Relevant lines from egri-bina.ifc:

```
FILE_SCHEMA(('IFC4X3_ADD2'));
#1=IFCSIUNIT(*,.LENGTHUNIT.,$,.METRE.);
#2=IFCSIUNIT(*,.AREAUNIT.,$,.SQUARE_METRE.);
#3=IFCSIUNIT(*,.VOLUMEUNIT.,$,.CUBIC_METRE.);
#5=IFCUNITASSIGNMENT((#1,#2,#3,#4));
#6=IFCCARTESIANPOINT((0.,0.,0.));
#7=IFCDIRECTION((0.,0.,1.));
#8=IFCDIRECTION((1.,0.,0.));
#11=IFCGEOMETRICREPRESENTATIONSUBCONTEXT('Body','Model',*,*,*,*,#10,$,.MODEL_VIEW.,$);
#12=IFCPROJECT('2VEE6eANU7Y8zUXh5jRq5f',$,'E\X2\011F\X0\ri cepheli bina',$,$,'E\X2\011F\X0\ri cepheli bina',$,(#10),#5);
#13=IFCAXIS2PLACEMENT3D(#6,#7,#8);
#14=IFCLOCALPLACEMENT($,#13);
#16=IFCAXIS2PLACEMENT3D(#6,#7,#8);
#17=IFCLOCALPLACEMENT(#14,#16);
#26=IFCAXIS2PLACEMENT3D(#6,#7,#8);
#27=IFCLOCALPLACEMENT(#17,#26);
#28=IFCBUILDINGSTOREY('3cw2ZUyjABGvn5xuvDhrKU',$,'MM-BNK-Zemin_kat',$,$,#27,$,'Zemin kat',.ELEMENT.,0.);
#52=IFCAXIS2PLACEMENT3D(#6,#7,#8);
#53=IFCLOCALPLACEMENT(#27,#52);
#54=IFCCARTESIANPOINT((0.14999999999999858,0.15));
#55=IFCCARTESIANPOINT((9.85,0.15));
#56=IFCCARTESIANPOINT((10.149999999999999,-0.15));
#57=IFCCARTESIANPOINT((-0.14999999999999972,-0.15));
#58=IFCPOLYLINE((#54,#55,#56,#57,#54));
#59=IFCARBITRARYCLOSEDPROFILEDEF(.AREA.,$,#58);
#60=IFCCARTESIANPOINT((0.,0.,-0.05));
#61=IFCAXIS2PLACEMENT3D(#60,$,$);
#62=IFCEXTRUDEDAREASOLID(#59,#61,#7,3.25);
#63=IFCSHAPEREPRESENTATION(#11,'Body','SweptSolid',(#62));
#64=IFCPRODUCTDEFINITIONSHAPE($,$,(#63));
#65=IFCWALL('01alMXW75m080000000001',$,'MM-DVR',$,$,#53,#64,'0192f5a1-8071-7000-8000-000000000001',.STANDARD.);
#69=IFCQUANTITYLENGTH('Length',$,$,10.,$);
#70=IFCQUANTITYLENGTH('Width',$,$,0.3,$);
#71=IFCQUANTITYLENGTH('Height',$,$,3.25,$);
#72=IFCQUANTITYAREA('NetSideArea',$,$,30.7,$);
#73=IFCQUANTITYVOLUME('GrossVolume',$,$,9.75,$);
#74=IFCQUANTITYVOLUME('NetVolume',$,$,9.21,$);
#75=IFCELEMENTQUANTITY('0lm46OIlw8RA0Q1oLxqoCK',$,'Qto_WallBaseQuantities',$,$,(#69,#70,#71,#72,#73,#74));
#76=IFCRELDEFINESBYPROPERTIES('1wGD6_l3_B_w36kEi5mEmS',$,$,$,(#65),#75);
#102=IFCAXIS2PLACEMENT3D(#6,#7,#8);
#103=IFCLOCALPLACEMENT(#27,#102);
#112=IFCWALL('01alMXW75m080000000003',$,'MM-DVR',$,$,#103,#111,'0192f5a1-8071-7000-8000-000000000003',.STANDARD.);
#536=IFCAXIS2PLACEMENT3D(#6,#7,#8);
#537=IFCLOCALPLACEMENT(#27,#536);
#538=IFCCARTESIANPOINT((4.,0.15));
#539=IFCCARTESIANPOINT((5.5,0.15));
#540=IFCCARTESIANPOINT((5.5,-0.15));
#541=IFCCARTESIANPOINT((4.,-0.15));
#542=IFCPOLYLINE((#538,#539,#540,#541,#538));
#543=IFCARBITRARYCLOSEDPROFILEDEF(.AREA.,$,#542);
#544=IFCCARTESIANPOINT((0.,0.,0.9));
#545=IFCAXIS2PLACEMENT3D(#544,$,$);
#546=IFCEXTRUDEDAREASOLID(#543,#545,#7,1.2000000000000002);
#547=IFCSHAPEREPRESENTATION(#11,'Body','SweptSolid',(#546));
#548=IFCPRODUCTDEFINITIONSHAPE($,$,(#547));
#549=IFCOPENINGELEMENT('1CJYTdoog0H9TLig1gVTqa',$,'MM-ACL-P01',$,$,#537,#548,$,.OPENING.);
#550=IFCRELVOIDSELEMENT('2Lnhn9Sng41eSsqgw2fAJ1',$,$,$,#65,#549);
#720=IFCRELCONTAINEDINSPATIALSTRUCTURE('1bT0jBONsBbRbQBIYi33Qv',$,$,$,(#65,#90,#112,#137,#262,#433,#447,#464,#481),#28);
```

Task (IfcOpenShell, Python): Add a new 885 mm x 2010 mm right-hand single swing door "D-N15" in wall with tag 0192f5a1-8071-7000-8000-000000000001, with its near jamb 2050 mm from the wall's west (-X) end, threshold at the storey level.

```python
import numpy as np
import ifcopenshell
import ifcopenshell.api.feature
import ifcopenshell.api.geometry
import ifcopenshell.api.pset
import ifcopenshell.api.root
import ifcopenshell.api.spatial
import ifcopenshell.geom
import ifcopenshell.util.element
import ifcopenshell.util.placement
import ifcopenshell.util.representation
import ifcopenshell.util.shape
import ifcopenshell.util.unit

model = ifcopenshell.open("egri-bina.ifc")
unit_scale = ifcopenshell.util.unit.calculate_unit_scale(model)
area_scale = ifcopenshell.util.unit.calculate_unit_scale(model, "AREAUNIT")
volume_scale = ifcopenshell.util.unit.calculate_unit_scale(model, "VOLUMEUNIT")
settings = ifcopenshell.geom.settings()


def volume(element):
    """Net volume in cubic metres, openings subtracted."""
    shape = ifcopenshell.geom.create_shape(settings, element)
    return ifcopenshell.util.shape.get_volume(shape.geometry)


wall = model.by_guid("01alMXW75m080000000001")
storey = ifcopenshell.util.element.get_container(wall, ifc_class="IfcBuildingStorey")
context = ifcopenshell.util.representation.get_context(model, "Model", "Body", "MODEL_VIEW")
before = volume(wall)

width, height, from_end, sill = 0.885, 2.01, 2.05, 0.0  # metres

# The wall runs along its own X axis, and the end named is its -X end.
wall_shape = ifcopenshell.geom.create_shape(settings, wall)
x, y, z = ifcopenshell.util.shape.get_vertices(wall_shape.geometry).T
start = x.min() + from_end
face, thickness = float(y.min()), float(y.max() - y.min())
wall_matrix = ifcopenshell.util.placement.get_local_placement(wall.ObjectPlacement)
level = ifcopenshell.util.placement.get_local_placement(storey.ObjectPlacement)[2, 3]


def in_wall(x, y):
    """Placement at x, y metres in the wall's axes, at sill height."""
    matrix = wall_matrix.copy()
    matrix[:, 3] = wall_matrix @ np.array([x / unit_scale, y / unit_scale, 0.0, 1.0])
    matrix[2, 3] = level + sill / unit_scale
    return matrix


# Opening: a box that overshoots both wall faces by 50 mm.
opening = ifcopenshell.api.root.create_entity(model, ifc_class="IfcOpeningElement", predefined_type="OPENING")
box = ifcopenshell.api.geometry.add_wall_representation(
    model, context=context, length=width, height=height, thickness=thickness + 0.1
)
ifcopenshell.api.geometry.assign_representation(model, product=opening, representation=box)
ifcopenshell.api.geometry.edit_object_placement(model, product=opening, matrix=in_wall(start, face - 0.05), is_si=False)
ifcopenshell.api.feature.add_feature(model, feature=opening, element=wall)

door = ifcopenshell.api.root.create_entity(model, ifc_class="IfcDoor", name="D-N15", predefined_type="DOOR")
door.OverallWidth, door.OverallHeight = width / unit_scale, height / unit_scale
door.OperationType = "SINGLE_SWING_RIGHT"
body = ifcopenshell.api.geometry.add_door_representation(
    model,
    context=context,
    overall_width=door.OverallWidth,
    overall_height=door.OverallHeight,
    operation_type="SINGLE_SWING_RIGHT",
    lining_properties={"LiningDepth": thickness / unit_scale, "ThresholdDepth": thickness / unit_scale},
)
ifcopenshell.api.geometry.assign_representation(model, product=door, representation=body)
ifcopenshell.api.spatial.assign_container(model, products=[door], relating_structure=storey)
ifcopenshell.api.feature.add_filling(model, opening=opening, element=door)

# The lining spans the wall, so the door starts at the wall face.
ifcopenshell.api.geometry.edit_object_placement(model, product=door, matrix=in_wall(start, face), is_si=False)

after = volume(wall)

# Update the wall's stored quantities.
qto = model.by_id(ifcopenshell.util.element.get_pset(wall, "Qto_WallBaseQuantities", should_inherit=False)["id"])
ifcopenshell.api.pset.edit_qto(model, qto=qto, properties={
    "NetSideArea": after / thickness / area_scale,
    "NetVolume": after / volume_scale,
})

print(f"wall volume {before:.3f} -> {after:.3f} m3")

model.write("egri-bina_edited.ifc")
```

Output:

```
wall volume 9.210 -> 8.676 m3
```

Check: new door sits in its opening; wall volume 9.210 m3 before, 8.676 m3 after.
